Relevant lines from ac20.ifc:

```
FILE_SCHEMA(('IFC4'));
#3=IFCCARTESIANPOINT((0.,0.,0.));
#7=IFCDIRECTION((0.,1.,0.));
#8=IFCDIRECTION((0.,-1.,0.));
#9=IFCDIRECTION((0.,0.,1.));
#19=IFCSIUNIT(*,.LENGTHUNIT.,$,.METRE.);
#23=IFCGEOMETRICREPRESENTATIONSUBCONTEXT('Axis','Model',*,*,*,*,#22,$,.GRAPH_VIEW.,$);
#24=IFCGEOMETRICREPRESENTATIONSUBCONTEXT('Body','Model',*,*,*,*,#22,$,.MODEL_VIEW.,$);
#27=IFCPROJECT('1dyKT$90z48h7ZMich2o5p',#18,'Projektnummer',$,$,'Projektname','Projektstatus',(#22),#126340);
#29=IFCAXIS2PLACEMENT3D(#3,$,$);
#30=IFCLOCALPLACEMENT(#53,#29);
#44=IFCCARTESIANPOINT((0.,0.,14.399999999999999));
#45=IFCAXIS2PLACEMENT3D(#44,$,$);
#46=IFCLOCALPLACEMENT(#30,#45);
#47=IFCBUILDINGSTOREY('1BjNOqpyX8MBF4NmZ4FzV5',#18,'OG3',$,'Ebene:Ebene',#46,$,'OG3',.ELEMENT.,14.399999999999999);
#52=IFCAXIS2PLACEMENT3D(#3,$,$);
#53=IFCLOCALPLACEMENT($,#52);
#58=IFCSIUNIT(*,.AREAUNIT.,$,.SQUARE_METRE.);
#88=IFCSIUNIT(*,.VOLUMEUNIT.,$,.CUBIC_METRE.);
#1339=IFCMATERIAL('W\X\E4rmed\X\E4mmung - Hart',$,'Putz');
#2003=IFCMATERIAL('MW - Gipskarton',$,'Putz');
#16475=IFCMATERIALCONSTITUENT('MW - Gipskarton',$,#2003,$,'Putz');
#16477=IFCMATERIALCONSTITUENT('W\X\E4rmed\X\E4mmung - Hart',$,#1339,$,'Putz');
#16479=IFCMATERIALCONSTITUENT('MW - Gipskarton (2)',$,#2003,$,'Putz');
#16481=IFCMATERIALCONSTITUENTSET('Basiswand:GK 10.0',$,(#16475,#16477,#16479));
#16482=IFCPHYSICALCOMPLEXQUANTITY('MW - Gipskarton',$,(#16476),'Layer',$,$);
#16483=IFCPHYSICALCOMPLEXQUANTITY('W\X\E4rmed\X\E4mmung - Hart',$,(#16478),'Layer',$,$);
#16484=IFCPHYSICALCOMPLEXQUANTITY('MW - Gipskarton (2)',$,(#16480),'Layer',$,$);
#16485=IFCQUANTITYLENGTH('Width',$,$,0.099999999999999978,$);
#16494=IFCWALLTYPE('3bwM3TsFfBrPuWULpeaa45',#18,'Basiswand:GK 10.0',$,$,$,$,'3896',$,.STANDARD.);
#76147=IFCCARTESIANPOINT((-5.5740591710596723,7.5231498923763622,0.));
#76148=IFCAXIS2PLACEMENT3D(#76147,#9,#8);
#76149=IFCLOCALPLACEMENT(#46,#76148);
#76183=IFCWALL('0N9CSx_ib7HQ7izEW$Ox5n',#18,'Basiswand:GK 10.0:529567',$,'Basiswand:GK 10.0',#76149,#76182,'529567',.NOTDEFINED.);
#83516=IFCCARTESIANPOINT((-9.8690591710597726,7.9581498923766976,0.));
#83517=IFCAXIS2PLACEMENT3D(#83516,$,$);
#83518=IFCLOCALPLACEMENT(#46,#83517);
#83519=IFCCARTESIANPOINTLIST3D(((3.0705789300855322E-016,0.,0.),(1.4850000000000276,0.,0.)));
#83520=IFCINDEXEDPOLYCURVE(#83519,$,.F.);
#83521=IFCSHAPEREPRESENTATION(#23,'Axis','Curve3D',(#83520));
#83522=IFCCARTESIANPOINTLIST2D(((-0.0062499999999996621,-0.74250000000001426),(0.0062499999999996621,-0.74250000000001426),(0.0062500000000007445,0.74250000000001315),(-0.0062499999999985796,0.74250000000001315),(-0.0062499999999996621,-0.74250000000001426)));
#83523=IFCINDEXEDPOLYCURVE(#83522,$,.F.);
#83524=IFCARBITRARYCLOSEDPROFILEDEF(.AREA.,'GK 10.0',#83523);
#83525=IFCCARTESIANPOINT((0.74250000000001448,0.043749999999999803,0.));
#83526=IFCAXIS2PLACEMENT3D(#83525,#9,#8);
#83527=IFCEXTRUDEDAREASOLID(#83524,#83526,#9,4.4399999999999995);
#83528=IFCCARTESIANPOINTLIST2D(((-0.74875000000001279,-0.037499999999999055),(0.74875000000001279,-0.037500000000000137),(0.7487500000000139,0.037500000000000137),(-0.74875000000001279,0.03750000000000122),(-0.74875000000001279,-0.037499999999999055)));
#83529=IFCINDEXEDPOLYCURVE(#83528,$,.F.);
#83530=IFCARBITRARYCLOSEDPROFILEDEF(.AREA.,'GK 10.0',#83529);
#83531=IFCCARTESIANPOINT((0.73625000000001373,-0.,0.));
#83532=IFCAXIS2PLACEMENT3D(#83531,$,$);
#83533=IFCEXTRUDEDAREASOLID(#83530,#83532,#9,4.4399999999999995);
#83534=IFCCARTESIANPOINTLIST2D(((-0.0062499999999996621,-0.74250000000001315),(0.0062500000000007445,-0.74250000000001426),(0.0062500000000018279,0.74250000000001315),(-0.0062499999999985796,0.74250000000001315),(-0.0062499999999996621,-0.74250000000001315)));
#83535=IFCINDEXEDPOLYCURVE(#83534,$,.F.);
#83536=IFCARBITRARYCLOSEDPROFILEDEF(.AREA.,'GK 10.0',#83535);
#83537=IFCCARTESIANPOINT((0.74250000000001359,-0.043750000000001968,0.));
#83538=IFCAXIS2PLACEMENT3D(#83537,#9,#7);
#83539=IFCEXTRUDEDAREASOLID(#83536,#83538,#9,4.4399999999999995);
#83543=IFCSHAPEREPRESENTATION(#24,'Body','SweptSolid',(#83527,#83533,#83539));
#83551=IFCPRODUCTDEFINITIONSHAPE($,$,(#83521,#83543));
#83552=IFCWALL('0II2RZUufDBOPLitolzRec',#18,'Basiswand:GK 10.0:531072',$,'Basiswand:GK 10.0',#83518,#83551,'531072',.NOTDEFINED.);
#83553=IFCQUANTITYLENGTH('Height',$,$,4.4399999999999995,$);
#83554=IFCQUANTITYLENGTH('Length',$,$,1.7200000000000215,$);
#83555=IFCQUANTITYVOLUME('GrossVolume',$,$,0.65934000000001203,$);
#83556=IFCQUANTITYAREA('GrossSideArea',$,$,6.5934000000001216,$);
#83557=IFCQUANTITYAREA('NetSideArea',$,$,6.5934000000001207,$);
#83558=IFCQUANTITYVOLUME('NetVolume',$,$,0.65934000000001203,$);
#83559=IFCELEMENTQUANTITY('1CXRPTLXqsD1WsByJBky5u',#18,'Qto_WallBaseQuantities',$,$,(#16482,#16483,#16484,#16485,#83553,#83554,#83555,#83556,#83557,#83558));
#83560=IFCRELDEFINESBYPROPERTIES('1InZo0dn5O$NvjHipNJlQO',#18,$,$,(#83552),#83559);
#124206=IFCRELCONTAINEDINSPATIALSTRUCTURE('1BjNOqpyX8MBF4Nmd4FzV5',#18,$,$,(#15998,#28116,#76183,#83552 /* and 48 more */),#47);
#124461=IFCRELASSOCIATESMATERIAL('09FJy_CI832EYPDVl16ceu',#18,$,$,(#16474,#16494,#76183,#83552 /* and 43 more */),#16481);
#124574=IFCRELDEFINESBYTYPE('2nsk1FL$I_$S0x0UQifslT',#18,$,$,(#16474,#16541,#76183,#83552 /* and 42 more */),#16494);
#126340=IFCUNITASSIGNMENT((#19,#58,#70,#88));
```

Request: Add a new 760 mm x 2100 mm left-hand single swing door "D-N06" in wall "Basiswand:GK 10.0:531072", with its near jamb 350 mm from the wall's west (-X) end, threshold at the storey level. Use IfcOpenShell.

```python
import numpy as np
import ifcopenshell
import ifcopenshell.api.feature
import ifcopenshell.api.geometry
import ifcopenshell.api.pset
import ifcopenshell.api.root
import ifcopenshell.api.spatial
import ifcopenshell.geom
import ifcopenshell.util.element
import ifcopenshell.util.placement
import ifcopenshell.util.representation
import ifcopenshell.util.shape
import ifcopenshell.util.unit

model = ifcopenshell.open("ac20.ifc")
unit_scale = ifcopenshell.util.unit.calculate_unit_scale(model)
area_scale = ifcopenshell.util.unit.calculate_unit_scale(model, "AREAUNIT")
volume_scale = ifcopenshell.util.unit.calculate_unit_scale(model, "VOLUMEUNIT")
settings = ifcopenshell.geom.settings()


def volume(element):
    """Net volume in cubic metres, openings subtracted."""
    shape = ifcopenshell.geom.create_shape(settings, element)
    return ifcopenshell.util.shape.get_volume(shape.geometry)


wall = model.by_guid("0II2RZUufDBOPLitolzRec")
storey = ifcopenshell.util.element.get_container(wall, ifc_class="IfcBuildingStorey")
context = ifcopenshell.util.representation.get_context(model, "Model", "Body", "MODEL_VIEW")
before = volume(wall)

width, height, from_end, sill = 0.76, 2.1, 0.35, 0.0  # metres

# The wall runs along its own X axis, and the end named is its -X end.
wall_shape = ifcopenshell.geom.create_shape(settings, wall)
x, y, z = ifcopenshell.util.shape.get_vertices(wall_shape.geometry).T
start = x.min() + from_end
face, thickness = float(y.min()), float(y.max() - y.min())
wall_matrix = ifcopenshell.util.placement.get_local_placement(wall.ObjectPlacement)
level = ifcopenshell.util.placement.get_local_placement(storey.ObjectPlacement)[2, 3]


def in_wall(x, y):
    """Placement at x, y metres in the wall's axes, at sill height."""
    matrix = wall_matrix.copy()
    matrix[:, 3] = wall_matrix @ np.array([x / unit_scale, y / unit_scale, 0.0, 1.0])
    matrix[2, 3] = level + sill / unit_scale
    return matrix


# Opening: a box that overshoots both wall faces by 50 mm.
opening = ifcopenshell.api.root.create_entity(model, ifc_class="IfcOpeningElement", predefined_type="OPENING")
box = ifcopenshell.api.geometry.add_wall_representation(
    model, context=context, length=width, height=height, thickness=thickness + 0.1
)
ifcopenshell.api.geometry.assign_representation(model, product=opening, representation=box)
ifcopenshell.api.geometry.edit_object_placement(model, product=opening, matrix=in_wall(start, face - 0.05), is_si=False)
ifcopenshell.api.feature.add_feature(model, feature=opening, element=wall)

door = ifcopenshell.api.root.create_entity(model, ifc_class="IfcDoor", name="D-N06", predefined_type="DOOR")
door.OverallWidth, door.OverallHeight = width / unit_scale, height / unit_scale
door.OperationType = "SINGLE_SWING_LEFT"
body = ifcopenshell.api.geometry.add_door_representation(
    model,
    context=context,
    overall_width=door.OverallWidth,
    overall_height=door.OverallHeight,
    operation_type="SINGLE_SWING_LEFT",
    lining_properties={"LiningDepth": thickness / unit_scale, "ThresholdDepth": thickness / unit_scale},
)
ifcopenshell.api.geometry.assign_representation(model, product=door, representation=body)
ifcopenshell.api.spatial.assign_container(model, products=[door], relating_structure=storey)
ifcopenshell.api.feature.add_filling(model, opening=opening, element=door)

# The lining spans the wall, so the door starts at the wall face.
ifcopenshell.api.geometry.edit_object_placement(model, product=door, matrix=in_wall(start, face), is_si=False)

after = volume(wall)

# Update the wall's stored quantities.
qto = model.by_id(ifcopenshell.util.element.get_pset(wall, "Qto_WallBaseQuantities", should_inherit=False)["id"])
ifcopenshell.api.pset.edit_qto(model, qto=qto, properties={
    "NetSideArea": after / thickness / area_scale,
    "NetVolume": after / volume_scale,
})

print(f"wall volume {before:.3f} -> {after:.3f} m3")

model.write("ac20_updated.ifc")
```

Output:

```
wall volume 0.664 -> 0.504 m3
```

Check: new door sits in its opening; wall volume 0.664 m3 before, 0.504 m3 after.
